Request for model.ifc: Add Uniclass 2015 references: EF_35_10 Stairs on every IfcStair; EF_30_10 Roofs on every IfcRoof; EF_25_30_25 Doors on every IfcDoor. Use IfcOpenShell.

First a look at what the model holds.

```python
import ifcopenshell

model = ifcopenshell.open("model.ifc")
print(model.schema)
print("classifications:", [c.Name for c in model.by_type("IfcClassification")])
for ifc_class in ("IfcDoor", "IfcRoof", "IfcStair", "IfcWall", "IfcWindow"):
    print(ifc_class, len(model.by_type(ifc_class)))
```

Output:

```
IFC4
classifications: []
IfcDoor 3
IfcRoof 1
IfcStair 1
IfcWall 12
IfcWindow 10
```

```python
import ifcopenshell
import ifcopenshell.api.classification

model = ifcopenshell.open("model.ifc")

system = ifcopenshell.api.classification.add_classification(model, classification="Uniclass 2015")

codes = {
    "IfcStair": ("EF_35_10", "Stairs"),
    "IfcRoof": ("EF_30_10", "Roofs"),
    "IfcDoor": ("EF_25_30_25", "Doors"),
}
for ifc_class, (code, name) in codes.items():
    products = model.by_type(ifc_class)
    ifcopenshell.api.classification.add_reference(
        model, products=products, classification=system, identification=code, name=name
    )
    print(code, len(products))

model.write("model_rev.ifc")
```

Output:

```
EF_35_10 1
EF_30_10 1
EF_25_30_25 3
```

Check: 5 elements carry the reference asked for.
